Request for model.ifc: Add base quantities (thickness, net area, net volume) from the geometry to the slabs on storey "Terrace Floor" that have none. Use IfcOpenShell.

First a look at what the model holds.

```python
import ifcopenshell
import ifcopenshell.util.element
import ifcopenshell.util.unit

model = ifcopenshell.open("model.ifc")
print(model.schema)
for unit_type in ("LENGTHUNIT", "AREAUNIT", "VOLUMEUNIT"):
    print(unit_type, ifcopenshell.util.unit.calculate_unit_scale(model, unit_type))
storey = next(s for s in model.by_type("IfcBuildingStorey") if s.Name == "Terrace Floor")
slabs = [e for e in ifcopenshell.util.element.get_decomposition(storey) if e.is_a("IfcSlab")]
for e in sorted(slabs, key=lambda e: e.id()):
    print(e.id(), e.is_a(), e.Name, list(ifcopenshell.util.element.get_psets(e, qtos_only=True)), sep=" | ")
```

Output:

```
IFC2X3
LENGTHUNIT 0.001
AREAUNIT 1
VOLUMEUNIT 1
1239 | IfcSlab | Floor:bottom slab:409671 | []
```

```python
import ifcopenshell
import ifcopenshell.api.pset
import ifcopenshell.geom
import ifcopenshell.util.element
import ifcopenshell.util.shape
import ifcopenshell.util.unit

model = ifcopenshell.open("model.ifc")
unit_scale = ifcopenshell.util.unit.calculate_unit_scale(model)
area_scale = ifcopenshell.util.unit.calculate_unit_scale(model, "AREAUNIT")
volume_scale = ifcopenshell.util.unit.calculate_unit_scale(model, "VOLUMEUNIT")
settings = ifcopenshell.geom.settings()

storey = next(s for s in model.by_type("IfcBuildingStorey") if s.Name == "Terrace Floor")
slabs = [e for e in ifcopenshell.util.element.get_decomposition(storey) if e.is_a("IfcSlab")]

for e in sorted(slabs, key=lambda e: e.id()):
    if ifcopenshell.util.element.get_psets(e, qtos_only=True, should_inherit=False):
        continue
    # Geometry comes back in metres, in the element's own axes.
    shape = ifcopenshell.geom.create_shape(settings, e)
    values = {
        "Width": ifcopenshell.util.shape.get_z(shape.geometry) / unit_scale,
        "NetArea": ifcopenshell.util.shape.get_footprint_area(shape.geometry) / area_scale,
        "NetVolume": ifcopenshell.util.shape.get_volume(shape.geometry) / volume_scale,
    }
    qto = ifcopenshell.api.pset.add_qto(model, product=e, name="BaseQuantities")
    ifcopenshell.api.pset.edit_qto(model, qto=qto, properties=values)
    print(e.id(), {k: round(v, 3) for k, v in values.items()})

model.write("model_updated.ifc")
```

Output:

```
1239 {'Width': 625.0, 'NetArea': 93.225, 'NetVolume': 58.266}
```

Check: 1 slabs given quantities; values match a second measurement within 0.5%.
